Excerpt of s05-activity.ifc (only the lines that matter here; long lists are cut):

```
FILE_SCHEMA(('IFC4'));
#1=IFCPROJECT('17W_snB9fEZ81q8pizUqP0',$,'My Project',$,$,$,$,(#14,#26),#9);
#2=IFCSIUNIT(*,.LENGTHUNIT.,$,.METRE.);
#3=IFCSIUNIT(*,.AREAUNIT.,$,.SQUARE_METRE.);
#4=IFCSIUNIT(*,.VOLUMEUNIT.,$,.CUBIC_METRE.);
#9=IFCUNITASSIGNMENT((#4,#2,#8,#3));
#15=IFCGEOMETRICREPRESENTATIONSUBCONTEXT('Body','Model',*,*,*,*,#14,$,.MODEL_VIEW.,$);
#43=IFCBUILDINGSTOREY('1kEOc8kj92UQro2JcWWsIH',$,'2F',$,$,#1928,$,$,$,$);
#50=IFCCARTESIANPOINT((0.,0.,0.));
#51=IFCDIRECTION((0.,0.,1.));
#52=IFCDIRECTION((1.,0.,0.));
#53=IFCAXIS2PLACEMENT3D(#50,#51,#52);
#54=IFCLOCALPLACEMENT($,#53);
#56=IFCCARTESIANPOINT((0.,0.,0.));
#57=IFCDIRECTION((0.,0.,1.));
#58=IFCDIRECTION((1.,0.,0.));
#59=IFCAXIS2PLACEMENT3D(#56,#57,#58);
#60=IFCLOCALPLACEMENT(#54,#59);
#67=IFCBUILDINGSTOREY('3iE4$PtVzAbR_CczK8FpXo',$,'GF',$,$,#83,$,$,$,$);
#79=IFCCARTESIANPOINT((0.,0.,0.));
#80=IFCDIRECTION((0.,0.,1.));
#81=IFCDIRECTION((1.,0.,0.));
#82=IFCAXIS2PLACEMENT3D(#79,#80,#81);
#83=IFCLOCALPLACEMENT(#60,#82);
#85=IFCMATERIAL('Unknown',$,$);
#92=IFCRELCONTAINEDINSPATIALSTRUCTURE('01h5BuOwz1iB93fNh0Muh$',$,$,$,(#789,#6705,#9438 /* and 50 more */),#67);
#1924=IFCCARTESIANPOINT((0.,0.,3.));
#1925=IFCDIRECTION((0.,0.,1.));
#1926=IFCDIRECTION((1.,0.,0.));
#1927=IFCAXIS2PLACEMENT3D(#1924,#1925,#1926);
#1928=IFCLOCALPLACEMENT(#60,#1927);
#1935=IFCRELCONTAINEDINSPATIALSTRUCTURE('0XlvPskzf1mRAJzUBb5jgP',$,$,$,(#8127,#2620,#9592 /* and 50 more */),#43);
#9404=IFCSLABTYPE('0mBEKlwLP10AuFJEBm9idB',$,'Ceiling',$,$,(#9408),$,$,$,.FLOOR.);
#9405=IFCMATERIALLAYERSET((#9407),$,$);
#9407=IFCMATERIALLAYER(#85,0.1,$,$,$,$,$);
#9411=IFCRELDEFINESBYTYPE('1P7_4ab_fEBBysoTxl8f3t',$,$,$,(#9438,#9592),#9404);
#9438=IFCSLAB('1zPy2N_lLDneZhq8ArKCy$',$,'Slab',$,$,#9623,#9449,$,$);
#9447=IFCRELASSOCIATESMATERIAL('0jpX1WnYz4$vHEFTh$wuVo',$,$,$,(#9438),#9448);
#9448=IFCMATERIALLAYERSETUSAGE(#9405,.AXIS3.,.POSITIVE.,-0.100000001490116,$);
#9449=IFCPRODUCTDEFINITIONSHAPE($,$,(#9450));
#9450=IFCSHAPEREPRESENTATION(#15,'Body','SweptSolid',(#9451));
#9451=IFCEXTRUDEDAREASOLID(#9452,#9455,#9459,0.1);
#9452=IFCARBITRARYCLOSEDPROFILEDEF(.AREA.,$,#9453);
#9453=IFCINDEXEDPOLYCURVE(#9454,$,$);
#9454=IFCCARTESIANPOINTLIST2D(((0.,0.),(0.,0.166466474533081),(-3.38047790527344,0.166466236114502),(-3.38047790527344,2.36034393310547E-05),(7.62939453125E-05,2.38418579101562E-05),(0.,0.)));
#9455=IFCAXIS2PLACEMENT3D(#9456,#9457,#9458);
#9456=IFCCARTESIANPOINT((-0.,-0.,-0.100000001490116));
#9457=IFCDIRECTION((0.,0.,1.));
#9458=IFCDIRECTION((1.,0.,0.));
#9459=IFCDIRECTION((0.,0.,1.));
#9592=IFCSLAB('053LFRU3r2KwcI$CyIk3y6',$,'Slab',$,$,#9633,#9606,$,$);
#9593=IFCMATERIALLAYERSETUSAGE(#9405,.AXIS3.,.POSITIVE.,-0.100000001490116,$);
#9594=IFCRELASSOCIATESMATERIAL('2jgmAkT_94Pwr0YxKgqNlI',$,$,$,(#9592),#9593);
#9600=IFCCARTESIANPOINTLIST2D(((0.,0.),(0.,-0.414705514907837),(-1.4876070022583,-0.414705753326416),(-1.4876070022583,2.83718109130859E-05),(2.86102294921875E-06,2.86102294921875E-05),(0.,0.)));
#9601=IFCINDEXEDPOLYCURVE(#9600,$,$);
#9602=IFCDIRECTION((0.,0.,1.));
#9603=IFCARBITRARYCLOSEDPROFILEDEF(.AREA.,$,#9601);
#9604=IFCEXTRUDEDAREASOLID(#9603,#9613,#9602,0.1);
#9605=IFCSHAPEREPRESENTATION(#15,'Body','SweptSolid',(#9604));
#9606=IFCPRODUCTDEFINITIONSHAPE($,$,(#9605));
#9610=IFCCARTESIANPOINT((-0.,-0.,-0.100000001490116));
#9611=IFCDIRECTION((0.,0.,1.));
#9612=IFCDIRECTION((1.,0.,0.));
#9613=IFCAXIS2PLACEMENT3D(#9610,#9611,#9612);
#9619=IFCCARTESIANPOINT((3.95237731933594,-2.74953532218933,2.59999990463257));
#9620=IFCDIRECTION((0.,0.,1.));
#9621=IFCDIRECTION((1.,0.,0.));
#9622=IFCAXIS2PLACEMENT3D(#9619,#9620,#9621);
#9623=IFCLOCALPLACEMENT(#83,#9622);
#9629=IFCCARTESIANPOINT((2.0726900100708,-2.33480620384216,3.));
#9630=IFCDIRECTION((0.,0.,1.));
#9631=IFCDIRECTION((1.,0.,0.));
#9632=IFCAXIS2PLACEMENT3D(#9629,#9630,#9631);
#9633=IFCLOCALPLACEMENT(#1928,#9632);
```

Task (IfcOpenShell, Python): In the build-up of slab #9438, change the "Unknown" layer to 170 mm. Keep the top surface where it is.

```python
import ifcopenshell
import ifcopenshell.util.element
import ifcopenshell.util.representation
import ifcopenshell.util.unit

model = ifcopenshell.open("s05-activity.ifc")
unit_scale = ifcopenshell.util.unit.calculate_unit_scale(model)

layer_set = model.by_id(9405)
layer = next(l for l in layer_set.MaterialLayers if l.Material and l.Material.Name == "Unknown")
change = 0.17 / unit_scale - layer.LayerThickness
layer.LayerThickness += change

# The layer set is shared, so every slab that uses it gets the new thickness.
slabs = [e for e in ifcopenshell.util.element.get_elements_by_material(model, layer_set) if e.is_a("IfcSlab")]
for slab in sorted(slabs, key=lambda e: e.id()):
    body = ifcopenshell.util.representation.get_representation(slab, "Model", "Body")
    solid = body.Items[0]
    old_depth = solid.Depth
    solid.Depth += change
    # Extruded upwards: lower the start of the extrusion so the top stays.
    x, y, z = solid.Position.Location.Coordinates
    solid.Position.Location = model.createIfcCartesianPoint((x, y, z - change))
    print(slab.id(), f"{old_depth:g} -> {solid.Depth:g}")

# The layers are counted up from the underside, which has moved.
for usage in {ifcopenshell.util.element.get_material(slab) for slab in slabs}:
    usage.OffsetFromReferenceLine -= change

model.write("s05-activity_updated.ifc")
```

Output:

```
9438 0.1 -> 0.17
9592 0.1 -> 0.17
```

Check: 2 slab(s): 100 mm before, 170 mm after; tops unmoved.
